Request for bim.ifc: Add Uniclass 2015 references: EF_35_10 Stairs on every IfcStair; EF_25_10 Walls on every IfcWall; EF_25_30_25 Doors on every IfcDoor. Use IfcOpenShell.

First a look at what the model holds.

```python
import ifcopenshell

model = ifcopenshell.open("bim.ifc")
print(model.schema)
print("classifications:", [c.Name for c in model.by_type("IfcClassification")])
for ifc_class in ("IfcDoor", "IfcRoof", "IfcStair", "IfcWall", "IfcWindow"):
    print(ifc_class, len(model.by_type(ifc_class)))
```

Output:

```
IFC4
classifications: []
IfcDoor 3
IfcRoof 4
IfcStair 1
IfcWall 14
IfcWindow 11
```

```python
import ifcopenshell
import ifcopenshell.api.classification

model = ifcopenshell.open("bim.ifc")

system = ifcopenshell.api.classification.add_classification(model, classification="Uniclass 2015")

codes = {
    "IfcStair": ("EF_35_10", "Stairs"),
    "IfcWall": ("EF_25_10", "Walls"),
    "IfcDoor": ("EF_25_30_25", "Doors"),
}
for ifc_class, (code, name) in codes.items():
    products = model.by_type(ifc_class)
    ifcopenshell.api.classification.add_reference(
        model, products=products, classification=system, identification=code, name=name
    )
    print(code, len(products))

model.write("bim_edited.ifc")
```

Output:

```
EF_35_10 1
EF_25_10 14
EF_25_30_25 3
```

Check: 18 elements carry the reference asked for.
